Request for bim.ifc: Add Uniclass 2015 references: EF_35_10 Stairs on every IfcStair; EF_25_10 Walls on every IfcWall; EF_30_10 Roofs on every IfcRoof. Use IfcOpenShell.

First a look at what the model holds.

```python
import ifcopenshell

model = ifcopenshell.open("bim.ifc")
print(model.schema)
print("classifications:", [c.Name for c in model.by_type("IfcClassification")])
for ifc_class in ("IfcDoor", "IfcRoof", "IfcStair", "IfcWall", "IfcWindow"):
    print(ifc_class, len(model.by_type(ifc_class)))
```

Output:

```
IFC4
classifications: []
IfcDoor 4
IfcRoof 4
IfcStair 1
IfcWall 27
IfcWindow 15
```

```python
import ifcopenshell
import ifcopenshell.api.classification

model = ifcopenshell.open("bim.ifc")

system = ifcopenshell.api.classification.add_classification(model, classification="Uniclass 2015")

codes = {
    "IfcStair": ("EF_35_10", "Stairs"),
    "IfcWall": ("EF_25_10", "Walls"),
    "IfcRoof": ("EF_30_10", "Roofs"),
}
for ifc_class, (code, name) in codes.items():
    products = model.by_type(ifc_class)
    ifcopenshell.api.classification.add_reference(
        model, products=products, classification=system, identification=code, name=name
    )
    print(code, len(products))

model.write("bim_edited.ifc")
```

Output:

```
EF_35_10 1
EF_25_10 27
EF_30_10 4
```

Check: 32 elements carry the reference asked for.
